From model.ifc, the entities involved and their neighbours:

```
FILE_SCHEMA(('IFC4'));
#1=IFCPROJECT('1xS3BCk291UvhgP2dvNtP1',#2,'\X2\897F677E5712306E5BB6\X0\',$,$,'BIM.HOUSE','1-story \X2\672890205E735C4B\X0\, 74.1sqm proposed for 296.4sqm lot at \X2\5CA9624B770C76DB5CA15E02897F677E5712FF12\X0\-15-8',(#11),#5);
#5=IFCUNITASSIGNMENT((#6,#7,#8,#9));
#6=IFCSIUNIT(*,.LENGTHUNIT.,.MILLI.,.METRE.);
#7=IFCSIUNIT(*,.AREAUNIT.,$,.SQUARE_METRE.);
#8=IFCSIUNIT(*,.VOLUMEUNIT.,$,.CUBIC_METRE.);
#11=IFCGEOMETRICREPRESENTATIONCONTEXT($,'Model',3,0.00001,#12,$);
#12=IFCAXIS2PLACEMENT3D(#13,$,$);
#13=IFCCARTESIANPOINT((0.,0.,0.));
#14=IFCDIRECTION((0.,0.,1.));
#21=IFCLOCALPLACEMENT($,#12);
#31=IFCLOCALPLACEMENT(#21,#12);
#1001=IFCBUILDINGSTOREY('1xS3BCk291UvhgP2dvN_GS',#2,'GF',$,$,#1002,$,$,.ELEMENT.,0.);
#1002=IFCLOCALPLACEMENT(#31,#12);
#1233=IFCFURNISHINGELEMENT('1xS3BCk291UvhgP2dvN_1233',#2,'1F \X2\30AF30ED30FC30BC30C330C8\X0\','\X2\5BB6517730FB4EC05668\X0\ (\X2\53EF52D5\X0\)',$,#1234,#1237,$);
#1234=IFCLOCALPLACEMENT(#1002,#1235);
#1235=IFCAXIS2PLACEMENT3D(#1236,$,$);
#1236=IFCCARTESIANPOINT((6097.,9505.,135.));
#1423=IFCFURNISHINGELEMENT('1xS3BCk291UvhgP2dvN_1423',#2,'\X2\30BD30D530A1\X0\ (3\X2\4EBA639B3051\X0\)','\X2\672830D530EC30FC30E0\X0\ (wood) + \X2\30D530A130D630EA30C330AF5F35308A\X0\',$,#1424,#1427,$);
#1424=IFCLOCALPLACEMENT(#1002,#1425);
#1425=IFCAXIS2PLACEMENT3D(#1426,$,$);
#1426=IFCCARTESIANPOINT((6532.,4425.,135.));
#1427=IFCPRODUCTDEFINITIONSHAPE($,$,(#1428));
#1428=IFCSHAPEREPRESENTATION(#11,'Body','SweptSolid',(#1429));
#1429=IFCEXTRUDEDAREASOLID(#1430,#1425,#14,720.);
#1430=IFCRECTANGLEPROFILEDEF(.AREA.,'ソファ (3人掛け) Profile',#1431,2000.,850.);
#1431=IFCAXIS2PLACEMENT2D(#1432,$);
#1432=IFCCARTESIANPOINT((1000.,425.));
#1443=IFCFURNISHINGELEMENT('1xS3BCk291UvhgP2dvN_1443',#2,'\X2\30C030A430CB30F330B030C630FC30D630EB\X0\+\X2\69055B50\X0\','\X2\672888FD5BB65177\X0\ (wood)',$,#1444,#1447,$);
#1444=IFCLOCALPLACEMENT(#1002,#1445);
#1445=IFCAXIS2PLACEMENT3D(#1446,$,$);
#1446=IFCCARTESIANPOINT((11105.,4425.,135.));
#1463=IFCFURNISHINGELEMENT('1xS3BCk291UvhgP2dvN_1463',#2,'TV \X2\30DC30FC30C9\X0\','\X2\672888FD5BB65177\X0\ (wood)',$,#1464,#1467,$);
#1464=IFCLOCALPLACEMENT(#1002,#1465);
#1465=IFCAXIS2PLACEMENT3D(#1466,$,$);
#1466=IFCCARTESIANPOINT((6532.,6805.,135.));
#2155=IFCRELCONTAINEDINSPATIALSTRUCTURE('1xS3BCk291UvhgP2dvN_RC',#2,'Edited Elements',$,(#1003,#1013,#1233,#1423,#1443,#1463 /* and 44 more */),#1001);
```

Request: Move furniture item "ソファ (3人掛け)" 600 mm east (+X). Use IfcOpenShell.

```python
import ifcopenshell
import ifcopenshell.api.geometry
import ifcopenshell.util.placement
import ifcopenshell.util.unit

model = ifcopenshell.open("model.ifc")
unit_scale = ifcopenshell.util.unit.calculate_unit_scale(model)

item = model.by_id(1423)
matrix = ifcopenshell.util.placement.get_local_placement(item.ObjectPlacement)
matrix[0, 3] += 0.6 / unit_scale
ifcopenshell.api.geometry.edit_object_placement(model, product=item, matrix=matrix, is_si=False)

print(ifcopenshell.util.placement.get_local_placement(item.ObjectPlacement).round(3) + 0.0)

model.write("model_edited.ifc")
```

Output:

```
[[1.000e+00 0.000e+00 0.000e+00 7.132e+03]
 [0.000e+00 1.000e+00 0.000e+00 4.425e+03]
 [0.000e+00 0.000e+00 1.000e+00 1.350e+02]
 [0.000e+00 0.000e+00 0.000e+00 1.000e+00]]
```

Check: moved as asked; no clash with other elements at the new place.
